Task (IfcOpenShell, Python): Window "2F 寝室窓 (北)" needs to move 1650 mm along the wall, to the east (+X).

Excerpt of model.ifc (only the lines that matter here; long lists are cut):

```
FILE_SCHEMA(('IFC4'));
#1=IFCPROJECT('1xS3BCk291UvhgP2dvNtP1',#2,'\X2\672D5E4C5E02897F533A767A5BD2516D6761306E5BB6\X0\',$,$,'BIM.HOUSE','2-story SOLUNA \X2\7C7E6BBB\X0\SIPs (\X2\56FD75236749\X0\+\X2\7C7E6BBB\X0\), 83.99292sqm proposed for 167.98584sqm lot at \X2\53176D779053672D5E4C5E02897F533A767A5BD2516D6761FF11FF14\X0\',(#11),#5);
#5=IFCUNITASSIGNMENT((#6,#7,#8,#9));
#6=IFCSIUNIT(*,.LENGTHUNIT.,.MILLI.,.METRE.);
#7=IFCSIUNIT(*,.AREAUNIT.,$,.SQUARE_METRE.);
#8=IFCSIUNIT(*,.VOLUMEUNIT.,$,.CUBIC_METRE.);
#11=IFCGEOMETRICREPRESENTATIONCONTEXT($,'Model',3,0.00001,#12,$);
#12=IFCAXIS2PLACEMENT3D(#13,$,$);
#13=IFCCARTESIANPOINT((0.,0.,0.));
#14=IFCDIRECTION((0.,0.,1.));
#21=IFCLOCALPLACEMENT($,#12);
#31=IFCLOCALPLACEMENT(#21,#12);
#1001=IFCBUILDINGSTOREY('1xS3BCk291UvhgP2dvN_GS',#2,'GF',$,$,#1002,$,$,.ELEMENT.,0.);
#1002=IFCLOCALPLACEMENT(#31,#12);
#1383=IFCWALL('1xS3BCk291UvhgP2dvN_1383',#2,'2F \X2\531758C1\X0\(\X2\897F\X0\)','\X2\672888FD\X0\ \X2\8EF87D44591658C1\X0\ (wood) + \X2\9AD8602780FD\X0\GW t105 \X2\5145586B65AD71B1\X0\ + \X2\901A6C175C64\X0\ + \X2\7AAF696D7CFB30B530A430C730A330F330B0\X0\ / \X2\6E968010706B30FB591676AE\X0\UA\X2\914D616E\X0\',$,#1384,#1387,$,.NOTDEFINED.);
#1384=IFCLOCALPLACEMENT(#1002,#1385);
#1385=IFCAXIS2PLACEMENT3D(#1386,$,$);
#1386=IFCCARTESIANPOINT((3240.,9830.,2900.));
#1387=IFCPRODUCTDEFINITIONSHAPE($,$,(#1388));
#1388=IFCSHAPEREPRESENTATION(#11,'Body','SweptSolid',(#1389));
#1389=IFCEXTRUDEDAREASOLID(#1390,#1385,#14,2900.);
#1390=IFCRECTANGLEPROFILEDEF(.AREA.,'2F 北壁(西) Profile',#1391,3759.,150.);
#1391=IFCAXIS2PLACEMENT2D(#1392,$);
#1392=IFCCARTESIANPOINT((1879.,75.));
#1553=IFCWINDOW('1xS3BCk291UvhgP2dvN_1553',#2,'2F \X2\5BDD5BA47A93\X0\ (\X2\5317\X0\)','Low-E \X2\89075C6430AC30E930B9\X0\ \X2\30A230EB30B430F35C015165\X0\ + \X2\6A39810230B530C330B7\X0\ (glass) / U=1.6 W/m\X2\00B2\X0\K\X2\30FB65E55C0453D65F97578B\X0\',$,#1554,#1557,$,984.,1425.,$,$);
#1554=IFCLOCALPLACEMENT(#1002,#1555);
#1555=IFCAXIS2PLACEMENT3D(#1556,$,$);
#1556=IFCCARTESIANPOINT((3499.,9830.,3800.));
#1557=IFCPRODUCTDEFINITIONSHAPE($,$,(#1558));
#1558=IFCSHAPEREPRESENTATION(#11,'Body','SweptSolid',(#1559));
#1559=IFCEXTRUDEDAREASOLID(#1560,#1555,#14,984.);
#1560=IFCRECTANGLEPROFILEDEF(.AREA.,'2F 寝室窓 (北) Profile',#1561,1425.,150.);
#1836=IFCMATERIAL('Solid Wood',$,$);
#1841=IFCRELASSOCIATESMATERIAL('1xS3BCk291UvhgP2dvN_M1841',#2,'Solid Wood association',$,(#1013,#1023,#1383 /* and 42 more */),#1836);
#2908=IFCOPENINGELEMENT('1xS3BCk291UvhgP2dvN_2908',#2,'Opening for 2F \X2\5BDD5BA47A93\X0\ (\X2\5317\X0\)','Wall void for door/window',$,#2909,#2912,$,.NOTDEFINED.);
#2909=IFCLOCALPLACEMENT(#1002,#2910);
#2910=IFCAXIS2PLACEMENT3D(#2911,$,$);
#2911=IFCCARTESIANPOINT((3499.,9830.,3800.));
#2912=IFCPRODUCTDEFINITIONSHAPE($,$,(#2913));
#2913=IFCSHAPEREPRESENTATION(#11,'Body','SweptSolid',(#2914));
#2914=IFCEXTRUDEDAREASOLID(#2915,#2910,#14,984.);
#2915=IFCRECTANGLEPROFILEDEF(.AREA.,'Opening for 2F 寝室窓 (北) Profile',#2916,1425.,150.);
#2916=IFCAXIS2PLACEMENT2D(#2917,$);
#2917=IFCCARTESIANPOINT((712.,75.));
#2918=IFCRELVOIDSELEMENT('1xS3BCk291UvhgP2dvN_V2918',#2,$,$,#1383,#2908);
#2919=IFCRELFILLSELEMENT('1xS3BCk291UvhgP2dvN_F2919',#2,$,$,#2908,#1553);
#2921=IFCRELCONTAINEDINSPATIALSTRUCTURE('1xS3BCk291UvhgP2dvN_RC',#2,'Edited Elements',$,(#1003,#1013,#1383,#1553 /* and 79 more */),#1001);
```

```python
import ifcopenshell
import ifcopenshell.api.geometry
import ifcopenshell.util.placement
import ifcopenshell.util.unit

model = ifcopenshell.open("model.ifc")
unit_scale = ifcopenshell.util.unit.calculate_unit_scale(model)

window = model.by_guid("1xS3BCk291UvhgP2dvN_1553")
opening = window.FillsVoids[0].RelatingOpeningElement
wall = opening.VoidsElements[0].RelatingBuildingElement

wall_matrix = ifcopenshell.util.placement.get_local_placement(wall.ObjectPlacement)
shift = wall_matrix[:3, 0] * 1.65 / unit_scale
before = ifcopenshell.util.placement.get_local_placement(window.ObjectPlacement)[:3, 3].copy()

# The window is not placed relative to its opening, so move both.
for product in (opening, window):
    matrix = ifcopenshell.util.placement.get_local_placement(product.ObjectPlacement)
    matrix[:3, 3] += shift
    ifcopenshell.api.geometry.edit_object_placement(model, product=product, matrix=matrix, is_si=False)

after = ifcopenshell.util.placement.get_local_placement(window.ObjectPlacement)[:3, 3]
print("window moved by", (after - before).round(3) + 0.0)

model.write("model_rev.ifc")
```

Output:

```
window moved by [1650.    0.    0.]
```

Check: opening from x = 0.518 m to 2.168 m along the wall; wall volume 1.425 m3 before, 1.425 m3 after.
